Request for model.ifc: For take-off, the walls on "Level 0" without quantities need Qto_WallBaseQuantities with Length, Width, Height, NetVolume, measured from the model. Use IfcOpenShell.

First a look at what the model holds.

```python
import ifcopenshell
import ifcopenshell.util.element
import ifcopenshell.util.unit

model = ifcopenshell.open("model.ifc")
print(model.schema)
for unit_type in ("LENGTHUNIT", "AREAUNIT", "VOLUMEUNIT"):
    print(unit_type, ifcopenshell.util.unit.calculate_unit_scale(model, unit_type))
storey = next(s for s in model.by_type("IfcBuildingStorey") if s.Name == "Level 0")
walls = [e for e in ifcopenshell.util.element.get_decomposition(storey) if e.is_a("IfcWall")]
for e in sorted(walls, key=lambda e: e.id()):
    print(e.id(), e.is_a(), e.Name, list(ifcopenshell.util.element.get_psets(e, qtos_only=True)), sep=" | ")
```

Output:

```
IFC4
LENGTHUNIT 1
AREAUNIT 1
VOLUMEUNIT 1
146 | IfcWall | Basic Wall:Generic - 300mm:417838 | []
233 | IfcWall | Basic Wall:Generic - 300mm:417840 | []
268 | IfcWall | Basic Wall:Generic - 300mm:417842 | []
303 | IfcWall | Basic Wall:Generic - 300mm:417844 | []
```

```python
import ifcopenshell
import ifcopenshell.api.pset
import ifcopenshell.geom
import ifcopenshell.util.element
import ifcopenshell.util.shape
import ifcopenshell.util.unit

model = ifcopenshell.open("model.ifc")
unit_scale = ifcopenshell.util.unit.calculate_unit_scale(model)
volume_scale = ifcopenshell.util.unit.calculate_unit_scale(model, "VOLUMEUNIT")
settings = ifcopenshell.geom.settings()

storey = next(s for s in model.by_type("IfcBuildingStorey") if s.Name == "Level 0")
walls = [e for e in ifcopenshell.util.element.get_decomposition(storey) if e.is_a("IfcWall")]

for e in sorted(walls, key=lambda e: e.id()):
    if ifcopenshell.util.element.get_psets(e, qtos_only=True, should_inherit=False):
        continue
    # Geometry comes back in metres, in the element's own axes.
    shape = ifcopenshell.geom.create_shape(settings, e)
    values = {
        "Length": ifcopenshell.util.shape.get_x(shape.geometry) / unit_scale,
        "Width": ifcopenshell.util.shape.get_y(shape.geometry) / unit_scale,
        "Height": ifcopenshell.util.shape.get_z(shape.geometry) / unit_scale,
        "NetVolume": ifcopenshell.util.shape.get_volume(shape.geometry) / volume_scale,
    }
    qto = ifcopenshell.api.pset.add_qto(model, product=e, name="Qto_WallBaseQuantities")
    ifcopenshell.api.pset.edit_qto(model, qto=qto, properties=values)
    print(e.id(), {k: round(v, 3) for k, v in values.items()})

model.write("model_rev.ifc")
```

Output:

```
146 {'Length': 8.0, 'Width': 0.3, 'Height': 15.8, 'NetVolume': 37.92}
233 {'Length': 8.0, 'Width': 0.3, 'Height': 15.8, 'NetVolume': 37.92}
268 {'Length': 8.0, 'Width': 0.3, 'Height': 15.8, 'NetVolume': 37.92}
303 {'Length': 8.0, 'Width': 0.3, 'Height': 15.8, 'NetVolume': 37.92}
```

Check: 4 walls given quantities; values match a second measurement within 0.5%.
